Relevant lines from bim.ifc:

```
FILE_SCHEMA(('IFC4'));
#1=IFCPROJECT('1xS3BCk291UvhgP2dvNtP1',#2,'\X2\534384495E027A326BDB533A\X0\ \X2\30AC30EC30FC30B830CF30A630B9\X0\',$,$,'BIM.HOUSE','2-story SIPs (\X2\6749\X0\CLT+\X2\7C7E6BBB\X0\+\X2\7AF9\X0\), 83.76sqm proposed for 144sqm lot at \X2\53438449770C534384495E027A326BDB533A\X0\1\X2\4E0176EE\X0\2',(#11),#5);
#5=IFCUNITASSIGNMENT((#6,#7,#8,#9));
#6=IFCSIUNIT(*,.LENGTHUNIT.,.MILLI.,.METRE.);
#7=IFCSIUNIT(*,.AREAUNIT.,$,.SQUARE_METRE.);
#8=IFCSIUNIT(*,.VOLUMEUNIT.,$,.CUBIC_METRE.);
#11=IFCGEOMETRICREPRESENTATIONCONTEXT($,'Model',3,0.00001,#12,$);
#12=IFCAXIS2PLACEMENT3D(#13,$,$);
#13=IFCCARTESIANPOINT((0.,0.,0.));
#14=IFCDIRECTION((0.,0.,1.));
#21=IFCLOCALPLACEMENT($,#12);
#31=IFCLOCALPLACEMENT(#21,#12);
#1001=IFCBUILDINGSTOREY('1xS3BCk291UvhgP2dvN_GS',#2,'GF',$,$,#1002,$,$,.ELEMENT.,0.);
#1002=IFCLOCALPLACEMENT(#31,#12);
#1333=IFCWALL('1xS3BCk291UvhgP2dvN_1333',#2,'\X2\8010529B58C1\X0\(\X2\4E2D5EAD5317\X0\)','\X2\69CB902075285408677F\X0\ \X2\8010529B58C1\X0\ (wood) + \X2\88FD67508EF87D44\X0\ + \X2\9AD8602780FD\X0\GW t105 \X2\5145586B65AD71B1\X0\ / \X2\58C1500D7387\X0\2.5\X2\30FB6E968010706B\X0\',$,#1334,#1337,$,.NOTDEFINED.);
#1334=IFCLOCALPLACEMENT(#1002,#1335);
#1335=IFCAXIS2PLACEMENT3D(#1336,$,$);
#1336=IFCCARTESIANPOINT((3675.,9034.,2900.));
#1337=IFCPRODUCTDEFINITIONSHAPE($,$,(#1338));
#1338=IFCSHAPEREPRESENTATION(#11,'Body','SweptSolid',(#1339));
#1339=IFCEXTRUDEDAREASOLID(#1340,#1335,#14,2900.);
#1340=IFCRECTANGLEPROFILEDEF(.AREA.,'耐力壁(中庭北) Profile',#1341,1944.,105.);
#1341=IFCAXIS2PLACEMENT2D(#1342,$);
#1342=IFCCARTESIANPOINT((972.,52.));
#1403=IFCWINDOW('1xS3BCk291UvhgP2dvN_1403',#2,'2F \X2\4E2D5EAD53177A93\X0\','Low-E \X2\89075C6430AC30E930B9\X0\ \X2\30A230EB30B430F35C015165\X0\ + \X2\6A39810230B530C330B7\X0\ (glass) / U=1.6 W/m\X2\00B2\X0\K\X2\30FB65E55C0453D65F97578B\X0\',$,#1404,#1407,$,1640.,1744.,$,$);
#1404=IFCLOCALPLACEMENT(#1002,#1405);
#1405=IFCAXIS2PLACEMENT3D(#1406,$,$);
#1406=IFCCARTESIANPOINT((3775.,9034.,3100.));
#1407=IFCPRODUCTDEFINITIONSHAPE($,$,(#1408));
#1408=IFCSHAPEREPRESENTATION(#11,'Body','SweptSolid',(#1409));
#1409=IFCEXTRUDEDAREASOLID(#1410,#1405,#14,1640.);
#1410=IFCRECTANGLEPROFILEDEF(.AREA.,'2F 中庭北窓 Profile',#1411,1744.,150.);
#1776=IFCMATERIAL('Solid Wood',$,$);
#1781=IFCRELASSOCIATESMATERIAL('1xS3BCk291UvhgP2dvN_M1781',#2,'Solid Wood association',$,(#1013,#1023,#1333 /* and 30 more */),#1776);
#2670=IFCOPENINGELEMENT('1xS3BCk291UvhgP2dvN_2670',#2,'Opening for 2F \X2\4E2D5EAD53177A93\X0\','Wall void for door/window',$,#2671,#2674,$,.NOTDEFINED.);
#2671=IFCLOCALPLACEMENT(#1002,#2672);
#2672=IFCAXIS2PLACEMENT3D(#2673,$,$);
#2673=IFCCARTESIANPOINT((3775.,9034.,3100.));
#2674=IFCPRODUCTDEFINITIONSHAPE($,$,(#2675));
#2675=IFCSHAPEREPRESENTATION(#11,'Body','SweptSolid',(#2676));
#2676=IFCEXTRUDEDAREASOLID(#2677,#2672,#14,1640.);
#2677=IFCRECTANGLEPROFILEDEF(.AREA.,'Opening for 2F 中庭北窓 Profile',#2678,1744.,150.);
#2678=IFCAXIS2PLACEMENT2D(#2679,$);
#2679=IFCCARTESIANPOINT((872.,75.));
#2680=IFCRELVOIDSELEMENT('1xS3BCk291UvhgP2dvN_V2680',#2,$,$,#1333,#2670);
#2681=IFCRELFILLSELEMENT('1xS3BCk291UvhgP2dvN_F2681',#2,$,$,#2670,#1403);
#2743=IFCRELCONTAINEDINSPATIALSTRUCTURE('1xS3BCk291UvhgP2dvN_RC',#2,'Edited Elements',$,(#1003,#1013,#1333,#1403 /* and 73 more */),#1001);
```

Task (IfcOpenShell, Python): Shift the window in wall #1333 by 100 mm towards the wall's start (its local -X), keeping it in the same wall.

```python
import ifcopenshell
import ifcopenshell.api.geometry
import ifcopenshell.util.placement
import ifcopenshell.util.unit

model = ifcopenshell.open("bim.ifc")
unit_scale = ifcopenshell.util.unit.calculate_unit_scale(model)

window = model.by_guid("1xS3BCk291UvhgP2dvN_1403")
opening = window.FillsVoids[0].RelatingOpeningElement
wall = opening.VoidsElements[0].RelatingBuildingElement

wall_matrix = ifcopenshell.util.placement.get_local_placement(wall.ObjectPlacement)
shift = wall_matrix[:3, 0] * -0.1 / unit_scale
before = ifcopenshell.util.placement.get_local_placement(window.ObjectPlacement)[:3, 3].copy()

# The window is not placed relative to its opening, so move both.
for product in (opening, window):
    matrix = ifcopenshell.util.placement.get_local_placement(product.ObjectPlacement)
    matrix[:3, 3] += shift
    ifcopenshell.api.geometry.edit_object_placement(model, product=product, matrix=matrix, is_si=False)

after = ifcopenshell.util.placement.get_local_placement(window.ObjectPlacement)[:3, 3]
print("window moved by", (after - before).round(3) + 0.0)

model.write("bim_v2.ifc")
```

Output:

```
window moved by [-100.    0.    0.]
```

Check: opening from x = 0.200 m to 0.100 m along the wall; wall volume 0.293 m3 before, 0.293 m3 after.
